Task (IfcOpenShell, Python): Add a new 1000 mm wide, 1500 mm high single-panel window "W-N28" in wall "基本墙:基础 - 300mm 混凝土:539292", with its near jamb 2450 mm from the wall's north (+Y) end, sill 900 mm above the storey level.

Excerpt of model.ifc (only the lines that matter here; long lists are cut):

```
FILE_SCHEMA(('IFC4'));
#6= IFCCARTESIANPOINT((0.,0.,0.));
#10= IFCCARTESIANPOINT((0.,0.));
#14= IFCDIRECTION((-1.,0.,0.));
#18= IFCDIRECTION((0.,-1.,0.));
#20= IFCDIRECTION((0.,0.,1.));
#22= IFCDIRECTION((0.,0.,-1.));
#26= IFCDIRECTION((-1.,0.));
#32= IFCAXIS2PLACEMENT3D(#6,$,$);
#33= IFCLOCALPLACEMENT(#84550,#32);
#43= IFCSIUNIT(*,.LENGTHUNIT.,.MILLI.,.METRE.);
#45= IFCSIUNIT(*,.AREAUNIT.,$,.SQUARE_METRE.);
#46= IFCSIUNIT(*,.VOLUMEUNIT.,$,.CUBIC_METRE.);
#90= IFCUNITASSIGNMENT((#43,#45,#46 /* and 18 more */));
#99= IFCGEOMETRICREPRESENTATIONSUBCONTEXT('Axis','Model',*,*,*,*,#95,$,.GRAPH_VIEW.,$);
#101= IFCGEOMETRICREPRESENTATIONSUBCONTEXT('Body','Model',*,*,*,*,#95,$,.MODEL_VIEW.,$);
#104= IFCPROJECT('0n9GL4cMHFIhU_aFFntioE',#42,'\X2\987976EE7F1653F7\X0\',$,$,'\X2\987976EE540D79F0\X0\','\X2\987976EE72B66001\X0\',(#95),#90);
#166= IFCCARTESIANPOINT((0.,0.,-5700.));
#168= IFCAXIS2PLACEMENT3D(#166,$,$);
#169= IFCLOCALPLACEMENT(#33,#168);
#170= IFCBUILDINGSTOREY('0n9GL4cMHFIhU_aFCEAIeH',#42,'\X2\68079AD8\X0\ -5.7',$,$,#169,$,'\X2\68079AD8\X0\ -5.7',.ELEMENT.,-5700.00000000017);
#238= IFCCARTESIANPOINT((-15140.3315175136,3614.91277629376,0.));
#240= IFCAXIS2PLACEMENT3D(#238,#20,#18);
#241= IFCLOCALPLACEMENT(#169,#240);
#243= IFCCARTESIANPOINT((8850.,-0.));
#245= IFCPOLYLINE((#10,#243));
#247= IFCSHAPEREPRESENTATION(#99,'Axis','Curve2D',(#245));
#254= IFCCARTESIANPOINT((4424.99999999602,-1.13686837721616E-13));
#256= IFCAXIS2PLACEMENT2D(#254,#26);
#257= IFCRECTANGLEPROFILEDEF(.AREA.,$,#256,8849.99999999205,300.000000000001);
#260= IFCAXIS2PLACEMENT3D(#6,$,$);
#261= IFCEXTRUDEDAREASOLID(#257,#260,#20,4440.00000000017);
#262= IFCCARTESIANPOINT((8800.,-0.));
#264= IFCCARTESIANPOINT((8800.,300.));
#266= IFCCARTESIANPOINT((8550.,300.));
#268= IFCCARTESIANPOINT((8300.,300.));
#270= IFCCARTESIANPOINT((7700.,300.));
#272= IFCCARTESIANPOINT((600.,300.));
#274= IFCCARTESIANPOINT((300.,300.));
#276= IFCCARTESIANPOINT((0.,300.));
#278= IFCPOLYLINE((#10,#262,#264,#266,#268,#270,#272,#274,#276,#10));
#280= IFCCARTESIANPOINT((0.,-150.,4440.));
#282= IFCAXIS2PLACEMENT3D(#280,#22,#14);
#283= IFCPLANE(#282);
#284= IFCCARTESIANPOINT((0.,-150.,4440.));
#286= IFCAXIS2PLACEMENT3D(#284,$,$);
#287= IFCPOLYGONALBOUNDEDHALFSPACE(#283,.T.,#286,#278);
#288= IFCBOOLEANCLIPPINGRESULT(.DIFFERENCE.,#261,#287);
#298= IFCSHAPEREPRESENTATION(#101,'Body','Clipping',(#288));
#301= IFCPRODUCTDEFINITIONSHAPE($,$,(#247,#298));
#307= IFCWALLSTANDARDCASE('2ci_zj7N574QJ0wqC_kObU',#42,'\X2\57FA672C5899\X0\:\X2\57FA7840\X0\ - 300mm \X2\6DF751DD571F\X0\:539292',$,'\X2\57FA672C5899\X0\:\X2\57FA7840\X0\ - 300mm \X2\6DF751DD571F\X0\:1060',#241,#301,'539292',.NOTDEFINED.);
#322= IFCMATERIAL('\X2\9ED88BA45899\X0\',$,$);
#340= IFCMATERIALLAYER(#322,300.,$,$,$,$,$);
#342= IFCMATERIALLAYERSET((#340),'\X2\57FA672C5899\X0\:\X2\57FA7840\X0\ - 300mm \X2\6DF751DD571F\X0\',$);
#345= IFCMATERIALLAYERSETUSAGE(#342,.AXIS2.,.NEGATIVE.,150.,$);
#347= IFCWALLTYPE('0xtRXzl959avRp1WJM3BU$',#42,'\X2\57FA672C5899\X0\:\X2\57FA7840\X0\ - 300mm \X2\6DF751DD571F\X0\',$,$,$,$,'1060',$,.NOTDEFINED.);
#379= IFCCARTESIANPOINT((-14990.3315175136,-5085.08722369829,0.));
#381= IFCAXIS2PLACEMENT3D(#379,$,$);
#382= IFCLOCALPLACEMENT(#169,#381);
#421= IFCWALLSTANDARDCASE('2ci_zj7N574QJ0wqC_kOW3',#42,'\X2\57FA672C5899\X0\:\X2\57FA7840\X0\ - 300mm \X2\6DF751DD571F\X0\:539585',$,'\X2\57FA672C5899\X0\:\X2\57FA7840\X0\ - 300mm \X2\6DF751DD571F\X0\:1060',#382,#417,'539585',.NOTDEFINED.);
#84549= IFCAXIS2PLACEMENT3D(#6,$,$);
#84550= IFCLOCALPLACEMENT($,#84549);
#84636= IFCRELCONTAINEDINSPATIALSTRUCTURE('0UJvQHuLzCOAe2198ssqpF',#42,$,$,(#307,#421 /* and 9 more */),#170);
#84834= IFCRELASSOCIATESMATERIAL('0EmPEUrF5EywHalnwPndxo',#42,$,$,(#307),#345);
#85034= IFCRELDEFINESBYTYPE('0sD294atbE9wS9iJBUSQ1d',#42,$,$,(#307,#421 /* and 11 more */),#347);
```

```python
import numpy as np
import ifcopenshell
import ifcopenshell.api.feature
import ifcopenshell.api.geometry
import ifcopenshell.api.root
import ifcopenshell.api.spatial
import ifcopenshell.geom
import ifcopenshell.util.element
import ifcopenshell.util.placement
import ifcopenshell.util.representation
import ifcopenshell.util.shape
import ifcopenshell.util.unit

model = ifcopenshell.open("model.ifc")
unit_scale = ifcopenshell.util.unit.calculate_unit_scale(model)
settings = ifcopenshell.geom.settings()


def volume(element):
    """Net volume in cubic metres, openings subtracted."""
    shape = ifcopenshell.geom.create_shape(settings, element)
    return ifcopenshell.util.shape.get_volume(shape.geometry)


wall = model.by_guid("2ci_zj7N574QJ0wqC_kObU")
storey = ifcopenshell.util.element.get_container(wall, ifc_class="IfcBuildingStorey")
context = ifcopenshell.util.representation.get_context(model, "Model", "Body", "MODEL_VIEW")
before = volume(wall)

width, height, from_end, sill = 1, 1.5, 2.45, 0.9  # metres

# The wall runs along its own X axis, and the end named is its -X end.
wall_shape = ifcopenshell.geom.create_shape(settings, wall)
x, y, z = ifcopenshell.util.shape.get_vertices(wall_shape.geometry).T
start = x.min() + from_end
face, thickness = float(y.min()), float(y.max() - y.min())
wall_matrix = ifcopenshell.util.placement.get_local_placement(wall.ObjectPlacement)
level = ifcopenshell.util.placement.get_local_placement(storey.ObjectPlacement)[2, 3]


def in_wall(x, y):
    """Placement at x, y metres in the wall's axes, at sill height."""
    matrix = wall_matrix.copy()
    matrix[:, 3] = wall_matrix @ np.array([x / unit_scale, y / unit_scale, 0.0, 1.0])
    matrix[2, 3] = level + sill / unit_scale
    return matrix


# Opening: a box that overshoots both wall faces by 50 mm.
opening = ifcopenshell.api.root.create_entity(model, ifc_class="IfcOpeningElement", predefined_type="OPENING")
box = ifcopenshell.api.geometry.add_wall_representation(
    model, context=context, length=width, height=height, thickness=thickness + 0.1
)
ifcopenshell.api.geometry.assign_representation(model, product=opening, representation=box)
ifcopenshell.api.geometry.edit_object_placement(model, product=opening, matrix=in_wall(start, face - 0.05), is_si=False)
ifcopenshell.api.feature.add_feature(model, feature=opening, element=wall)

window = ifcopenshell.api.root.create_entity(model, ifc_class="IfcWindow", name="W-N28", predefined_type="WINDOW")
window.OverallWidth, window.OverallHeight = width / unit_scale, height / unit_scale
window.PartitioningType = "SINGLE_PANEL"
body = ifcopenshell.api.geometry.add_window_representation(
    model,
    context=context,
    overall_width=window.OverallWidth,
    overall_height=window.OverallHeight,
    partition_type="SINGLE_PANEL",
)
ifcopenshell.api.geometry.assign_representation(model, product=window, representation=body)
ifcopenshell.api.spatial.assign_container(model, products=[window], relating_structure=storey)
ifcopenshell.api.feature.add_filling(model, opening=opening, element=window)

# Centre the window in the wall's thickness.
ifcopenshell.api.geometry.edit_object_placement(model, product=window, matrix=in_wall(start, face), is_si=False)
window_shape = ifcopenshell.geom.create_shape(settings, window)
depth = ifcopenshell.util.shape.get_vertices(window_shape.geometry)[:, 1]
offset = face + thickness / 2 - (depth.min() + depth.max()) / 2
ifcopenshell.api.geometry.edit_object_placement(model, product=window, matrix=in_wall(start, offset), is_si=False)

after = volume(wall)

print(f"wall volume {before:.3f} -> {after:.3f} m3")

model.write("model_v2.ifc")
```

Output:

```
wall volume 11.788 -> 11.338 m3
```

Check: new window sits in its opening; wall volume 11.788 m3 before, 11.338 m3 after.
